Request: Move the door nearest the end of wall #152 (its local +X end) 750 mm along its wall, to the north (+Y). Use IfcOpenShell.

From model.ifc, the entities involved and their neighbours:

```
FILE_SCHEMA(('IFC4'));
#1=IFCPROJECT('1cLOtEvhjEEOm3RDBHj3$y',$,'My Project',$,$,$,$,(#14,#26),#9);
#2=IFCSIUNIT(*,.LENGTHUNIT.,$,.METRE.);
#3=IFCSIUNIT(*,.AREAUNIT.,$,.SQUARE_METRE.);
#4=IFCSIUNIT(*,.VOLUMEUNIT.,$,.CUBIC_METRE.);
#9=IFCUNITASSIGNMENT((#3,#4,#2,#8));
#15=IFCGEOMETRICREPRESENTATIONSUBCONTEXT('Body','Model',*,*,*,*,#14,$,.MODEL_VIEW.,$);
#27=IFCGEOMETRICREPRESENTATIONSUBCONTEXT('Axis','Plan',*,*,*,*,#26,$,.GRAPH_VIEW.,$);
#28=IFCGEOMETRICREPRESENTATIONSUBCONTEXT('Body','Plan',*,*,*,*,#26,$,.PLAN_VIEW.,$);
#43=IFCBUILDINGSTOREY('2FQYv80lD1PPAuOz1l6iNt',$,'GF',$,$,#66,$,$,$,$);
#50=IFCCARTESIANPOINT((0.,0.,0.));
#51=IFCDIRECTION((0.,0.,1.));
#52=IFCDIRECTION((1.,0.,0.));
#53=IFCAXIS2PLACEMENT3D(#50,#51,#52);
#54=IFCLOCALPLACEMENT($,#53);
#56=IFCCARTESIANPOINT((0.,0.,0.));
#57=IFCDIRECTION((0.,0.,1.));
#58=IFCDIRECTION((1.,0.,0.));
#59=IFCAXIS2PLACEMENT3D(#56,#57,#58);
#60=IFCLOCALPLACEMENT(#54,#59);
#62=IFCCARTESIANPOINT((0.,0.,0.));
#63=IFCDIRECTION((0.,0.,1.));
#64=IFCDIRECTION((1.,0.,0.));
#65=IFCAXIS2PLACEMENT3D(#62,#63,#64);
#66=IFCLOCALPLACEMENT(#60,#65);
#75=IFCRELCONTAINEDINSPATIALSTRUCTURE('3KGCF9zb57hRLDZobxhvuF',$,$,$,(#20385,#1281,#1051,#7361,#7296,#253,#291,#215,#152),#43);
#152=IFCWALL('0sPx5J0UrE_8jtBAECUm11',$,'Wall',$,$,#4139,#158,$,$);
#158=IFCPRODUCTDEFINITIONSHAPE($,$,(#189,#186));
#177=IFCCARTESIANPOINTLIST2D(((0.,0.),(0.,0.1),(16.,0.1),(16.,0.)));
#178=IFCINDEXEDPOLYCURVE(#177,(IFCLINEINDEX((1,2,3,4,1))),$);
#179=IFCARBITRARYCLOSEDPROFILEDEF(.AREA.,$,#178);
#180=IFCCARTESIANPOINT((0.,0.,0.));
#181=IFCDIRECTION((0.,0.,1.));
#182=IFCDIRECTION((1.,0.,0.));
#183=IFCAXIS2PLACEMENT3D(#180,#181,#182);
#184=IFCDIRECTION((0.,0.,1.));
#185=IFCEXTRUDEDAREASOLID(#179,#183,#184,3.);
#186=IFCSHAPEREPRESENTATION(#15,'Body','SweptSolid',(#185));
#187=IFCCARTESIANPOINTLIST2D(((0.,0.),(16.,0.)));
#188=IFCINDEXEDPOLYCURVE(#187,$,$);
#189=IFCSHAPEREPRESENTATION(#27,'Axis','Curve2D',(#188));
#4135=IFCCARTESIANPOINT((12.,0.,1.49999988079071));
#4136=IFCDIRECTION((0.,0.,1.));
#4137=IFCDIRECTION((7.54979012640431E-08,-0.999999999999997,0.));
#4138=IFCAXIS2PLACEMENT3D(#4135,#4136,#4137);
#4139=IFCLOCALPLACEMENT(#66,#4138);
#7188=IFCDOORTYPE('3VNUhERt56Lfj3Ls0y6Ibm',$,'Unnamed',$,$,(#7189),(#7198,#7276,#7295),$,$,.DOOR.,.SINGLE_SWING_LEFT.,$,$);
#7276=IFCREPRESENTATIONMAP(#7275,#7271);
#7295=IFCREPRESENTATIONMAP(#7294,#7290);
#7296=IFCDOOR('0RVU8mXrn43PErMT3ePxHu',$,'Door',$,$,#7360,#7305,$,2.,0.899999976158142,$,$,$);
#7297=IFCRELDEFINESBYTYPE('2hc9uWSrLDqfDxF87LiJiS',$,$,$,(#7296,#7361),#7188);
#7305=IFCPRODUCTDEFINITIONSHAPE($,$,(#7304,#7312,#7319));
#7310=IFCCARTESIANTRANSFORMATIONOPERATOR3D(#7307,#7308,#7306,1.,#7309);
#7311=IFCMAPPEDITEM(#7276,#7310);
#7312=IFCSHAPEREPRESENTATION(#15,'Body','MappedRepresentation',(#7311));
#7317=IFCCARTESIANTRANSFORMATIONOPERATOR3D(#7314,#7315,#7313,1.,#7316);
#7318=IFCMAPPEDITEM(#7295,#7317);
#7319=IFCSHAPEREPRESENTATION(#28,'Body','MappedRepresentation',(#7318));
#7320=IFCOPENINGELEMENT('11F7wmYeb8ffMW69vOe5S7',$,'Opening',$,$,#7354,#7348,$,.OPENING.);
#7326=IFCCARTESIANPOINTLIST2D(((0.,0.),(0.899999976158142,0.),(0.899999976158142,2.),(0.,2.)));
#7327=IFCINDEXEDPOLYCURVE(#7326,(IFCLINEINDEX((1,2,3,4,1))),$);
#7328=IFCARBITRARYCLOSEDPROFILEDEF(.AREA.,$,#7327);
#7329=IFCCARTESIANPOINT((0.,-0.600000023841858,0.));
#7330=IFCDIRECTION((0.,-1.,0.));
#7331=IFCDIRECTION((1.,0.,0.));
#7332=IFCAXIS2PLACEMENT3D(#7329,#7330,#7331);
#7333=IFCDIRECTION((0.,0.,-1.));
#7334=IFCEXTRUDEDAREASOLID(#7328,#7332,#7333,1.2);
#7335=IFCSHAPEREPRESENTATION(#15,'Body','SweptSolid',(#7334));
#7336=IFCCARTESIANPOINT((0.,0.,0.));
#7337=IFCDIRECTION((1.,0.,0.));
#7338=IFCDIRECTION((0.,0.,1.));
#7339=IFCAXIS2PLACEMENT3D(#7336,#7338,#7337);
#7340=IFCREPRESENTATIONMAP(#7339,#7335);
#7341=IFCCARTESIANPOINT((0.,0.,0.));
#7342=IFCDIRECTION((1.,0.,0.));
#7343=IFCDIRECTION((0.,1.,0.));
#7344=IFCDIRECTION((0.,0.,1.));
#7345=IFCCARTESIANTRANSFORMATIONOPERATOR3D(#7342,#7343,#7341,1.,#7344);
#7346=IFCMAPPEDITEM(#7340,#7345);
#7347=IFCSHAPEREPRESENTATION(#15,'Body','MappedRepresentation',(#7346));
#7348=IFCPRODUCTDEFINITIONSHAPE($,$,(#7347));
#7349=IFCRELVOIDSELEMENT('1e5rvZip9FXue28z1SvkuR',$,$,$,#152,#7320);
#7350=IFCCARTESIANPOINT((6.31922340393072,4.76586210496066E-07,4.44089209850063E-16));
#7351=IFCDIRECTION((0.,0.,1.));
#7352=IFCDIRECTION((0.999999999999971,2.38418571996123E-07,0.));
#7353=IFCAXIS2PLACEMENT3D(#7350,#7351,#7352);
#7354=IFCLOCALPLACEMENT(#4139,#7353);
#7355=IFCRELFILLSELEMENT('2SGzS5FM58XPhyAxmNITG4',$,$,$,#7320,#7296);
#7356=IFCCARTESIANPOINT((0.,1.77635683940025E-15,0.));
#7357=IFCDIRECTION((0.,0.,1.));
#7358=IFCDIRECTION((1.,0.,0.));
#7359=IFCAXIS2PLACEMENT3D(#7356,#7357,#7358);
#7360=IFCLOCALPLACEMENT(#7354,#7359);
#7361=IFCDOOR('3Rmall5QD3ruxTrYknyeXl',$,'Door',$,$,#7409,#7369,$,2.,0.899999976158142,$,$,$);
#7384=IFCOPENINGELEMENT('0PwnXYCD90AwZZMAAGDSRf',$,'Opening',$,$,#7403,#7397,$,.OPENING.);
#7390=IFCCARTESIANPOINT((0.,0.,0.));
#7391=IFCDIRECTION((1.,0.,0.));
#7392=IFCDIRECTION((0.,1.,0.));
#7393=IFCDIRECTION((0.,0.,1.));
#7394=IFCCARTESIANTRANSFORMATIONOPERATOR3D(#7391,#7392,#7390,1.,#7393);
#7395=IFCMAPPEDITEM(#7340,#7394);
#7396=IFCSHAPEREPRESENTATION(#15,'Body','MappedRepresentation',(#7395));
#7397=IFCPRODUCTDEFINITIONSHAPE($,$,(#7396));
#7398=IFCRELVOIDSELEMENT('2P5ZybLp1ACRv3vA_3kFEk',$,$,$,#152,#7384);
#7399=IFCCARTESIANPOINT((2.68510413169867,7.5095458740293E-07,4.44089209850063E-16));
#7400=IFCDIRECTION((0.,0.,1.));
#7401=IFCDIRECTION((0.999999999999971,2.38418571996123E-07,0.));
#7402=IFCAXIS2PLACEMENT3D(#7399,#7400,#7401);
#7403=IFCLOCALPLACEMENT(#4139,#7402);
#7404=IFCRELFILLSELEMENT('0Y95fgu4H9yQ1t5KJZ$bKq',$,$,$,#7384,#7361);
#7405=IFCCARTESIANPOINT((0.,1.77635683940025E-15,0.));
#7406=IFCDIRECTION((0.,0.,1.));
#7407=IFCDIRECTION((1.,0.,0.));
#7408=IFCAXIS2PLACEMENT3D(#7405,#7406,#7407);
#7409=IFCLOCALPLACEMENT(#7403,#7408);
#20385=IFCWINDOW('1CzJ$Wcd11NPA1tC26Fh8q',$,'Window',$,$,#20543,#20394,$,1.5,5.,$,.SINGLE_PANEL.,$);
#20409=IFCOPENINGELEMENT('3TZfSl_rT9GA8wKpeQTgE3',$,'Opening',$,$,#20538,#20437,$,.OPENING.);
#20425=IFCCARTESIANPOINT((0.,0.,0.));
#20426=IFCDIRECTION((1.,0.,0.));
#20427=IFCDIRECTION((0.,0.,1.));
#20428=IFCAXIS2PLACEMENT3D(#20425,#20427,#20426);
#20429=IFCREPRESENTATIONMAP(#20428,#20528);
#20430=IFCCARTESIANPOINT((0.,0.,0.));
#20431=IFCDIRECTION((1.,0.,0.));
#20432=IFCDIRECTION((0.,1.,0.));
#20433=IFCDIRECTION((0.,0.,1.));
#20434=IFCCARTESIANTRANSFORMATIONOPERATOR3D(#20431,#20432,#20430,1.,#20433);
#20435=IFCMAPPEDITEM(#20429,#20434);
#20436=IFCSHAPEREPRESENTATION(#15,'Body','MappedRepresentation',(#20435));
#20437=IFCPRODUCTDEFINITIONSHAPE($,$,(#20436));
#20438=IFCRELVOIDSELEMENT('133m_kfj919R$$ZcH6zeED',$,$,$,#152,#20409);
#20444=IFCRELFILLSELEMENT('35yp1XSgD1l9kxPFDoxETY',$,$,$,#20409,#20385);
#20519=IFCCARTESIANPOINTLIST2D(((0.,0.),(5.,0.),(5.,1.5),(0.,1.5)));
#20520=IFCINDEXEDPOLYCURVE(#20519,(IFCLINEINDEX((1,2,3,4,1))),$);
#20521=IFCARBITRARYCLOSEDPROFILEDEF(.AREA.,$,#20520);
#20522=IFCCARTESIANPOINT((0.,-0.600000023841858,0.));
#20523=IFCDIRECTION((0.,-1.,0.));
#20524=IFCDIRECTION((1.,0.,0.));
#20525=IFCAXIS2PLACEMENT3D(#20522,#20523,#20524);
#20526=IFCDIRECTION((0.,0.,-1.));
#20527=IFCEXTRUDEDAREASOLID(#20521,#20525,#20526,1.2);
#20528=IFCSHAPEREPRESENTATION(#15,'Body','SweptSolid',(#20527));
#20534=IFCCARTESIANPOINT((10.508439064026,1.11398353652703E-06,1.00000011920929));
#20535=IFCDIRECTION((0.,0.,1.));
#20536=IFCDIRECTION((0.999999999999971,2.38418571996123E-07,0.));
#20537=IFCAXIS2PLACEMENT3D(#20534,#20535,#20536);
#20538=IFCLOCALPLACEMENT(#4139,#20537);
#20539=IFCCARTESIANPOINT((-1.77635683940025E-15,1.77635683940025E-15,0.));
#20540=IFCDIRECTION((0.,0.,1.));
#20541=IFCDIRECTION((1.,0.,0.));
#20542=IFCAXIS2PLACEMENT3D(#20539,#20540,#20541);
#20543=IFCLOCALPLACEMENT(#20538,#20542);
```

```python
import ifcopenshell
import ifcopenshell.api.geometry
import ifcopenshell.util.placement
import ifcopenshell.util.unit

model = ifcopenshell.open("model.ifc")
unit_scale = ifcopenshell.util.unit.calculate_unit_scale(model)

door = model.by_guid("0RVU8mXrn43PErMT3ePxHu")
opening = door.FillsVoids[0].RelatingOpeningElement
wall = opening.VoidsElements[0].RelatingBuildingElement

wall_matrix = ifcopenshell.util.placement.get_local_placement(wall.ObjectPlacement)
shift = wall_matrix[:3, 0] * -0.75 / unit_scale
before = ifcopenshell.util.placement.get_local_placement(door.ObjectPlacement)[:3, 3].copy()

# The door is placed relative to its opening, so it follows when the opening moves.
matrix = ifcopenshell.util.placement.get_local_placement(opening.ObjectPlacement)
matrix[:3, 3] += shift
ifcopenshell.api.geometry.edit_object_placement(
    model, product=opening, matrix=matrix, is_si=False, should_transform_children=True
)

after = ifcopenshell.util.placement.get_local_placement(door.ObjectPlacement)[:3, 3]
print("door moved by", (after - before).round(3) + 0.0)

model.write("model_v2.ifc")
```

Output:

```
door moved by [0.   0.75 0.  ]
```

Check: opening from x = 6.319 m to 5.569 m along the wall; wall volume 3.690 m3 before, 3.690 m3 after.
